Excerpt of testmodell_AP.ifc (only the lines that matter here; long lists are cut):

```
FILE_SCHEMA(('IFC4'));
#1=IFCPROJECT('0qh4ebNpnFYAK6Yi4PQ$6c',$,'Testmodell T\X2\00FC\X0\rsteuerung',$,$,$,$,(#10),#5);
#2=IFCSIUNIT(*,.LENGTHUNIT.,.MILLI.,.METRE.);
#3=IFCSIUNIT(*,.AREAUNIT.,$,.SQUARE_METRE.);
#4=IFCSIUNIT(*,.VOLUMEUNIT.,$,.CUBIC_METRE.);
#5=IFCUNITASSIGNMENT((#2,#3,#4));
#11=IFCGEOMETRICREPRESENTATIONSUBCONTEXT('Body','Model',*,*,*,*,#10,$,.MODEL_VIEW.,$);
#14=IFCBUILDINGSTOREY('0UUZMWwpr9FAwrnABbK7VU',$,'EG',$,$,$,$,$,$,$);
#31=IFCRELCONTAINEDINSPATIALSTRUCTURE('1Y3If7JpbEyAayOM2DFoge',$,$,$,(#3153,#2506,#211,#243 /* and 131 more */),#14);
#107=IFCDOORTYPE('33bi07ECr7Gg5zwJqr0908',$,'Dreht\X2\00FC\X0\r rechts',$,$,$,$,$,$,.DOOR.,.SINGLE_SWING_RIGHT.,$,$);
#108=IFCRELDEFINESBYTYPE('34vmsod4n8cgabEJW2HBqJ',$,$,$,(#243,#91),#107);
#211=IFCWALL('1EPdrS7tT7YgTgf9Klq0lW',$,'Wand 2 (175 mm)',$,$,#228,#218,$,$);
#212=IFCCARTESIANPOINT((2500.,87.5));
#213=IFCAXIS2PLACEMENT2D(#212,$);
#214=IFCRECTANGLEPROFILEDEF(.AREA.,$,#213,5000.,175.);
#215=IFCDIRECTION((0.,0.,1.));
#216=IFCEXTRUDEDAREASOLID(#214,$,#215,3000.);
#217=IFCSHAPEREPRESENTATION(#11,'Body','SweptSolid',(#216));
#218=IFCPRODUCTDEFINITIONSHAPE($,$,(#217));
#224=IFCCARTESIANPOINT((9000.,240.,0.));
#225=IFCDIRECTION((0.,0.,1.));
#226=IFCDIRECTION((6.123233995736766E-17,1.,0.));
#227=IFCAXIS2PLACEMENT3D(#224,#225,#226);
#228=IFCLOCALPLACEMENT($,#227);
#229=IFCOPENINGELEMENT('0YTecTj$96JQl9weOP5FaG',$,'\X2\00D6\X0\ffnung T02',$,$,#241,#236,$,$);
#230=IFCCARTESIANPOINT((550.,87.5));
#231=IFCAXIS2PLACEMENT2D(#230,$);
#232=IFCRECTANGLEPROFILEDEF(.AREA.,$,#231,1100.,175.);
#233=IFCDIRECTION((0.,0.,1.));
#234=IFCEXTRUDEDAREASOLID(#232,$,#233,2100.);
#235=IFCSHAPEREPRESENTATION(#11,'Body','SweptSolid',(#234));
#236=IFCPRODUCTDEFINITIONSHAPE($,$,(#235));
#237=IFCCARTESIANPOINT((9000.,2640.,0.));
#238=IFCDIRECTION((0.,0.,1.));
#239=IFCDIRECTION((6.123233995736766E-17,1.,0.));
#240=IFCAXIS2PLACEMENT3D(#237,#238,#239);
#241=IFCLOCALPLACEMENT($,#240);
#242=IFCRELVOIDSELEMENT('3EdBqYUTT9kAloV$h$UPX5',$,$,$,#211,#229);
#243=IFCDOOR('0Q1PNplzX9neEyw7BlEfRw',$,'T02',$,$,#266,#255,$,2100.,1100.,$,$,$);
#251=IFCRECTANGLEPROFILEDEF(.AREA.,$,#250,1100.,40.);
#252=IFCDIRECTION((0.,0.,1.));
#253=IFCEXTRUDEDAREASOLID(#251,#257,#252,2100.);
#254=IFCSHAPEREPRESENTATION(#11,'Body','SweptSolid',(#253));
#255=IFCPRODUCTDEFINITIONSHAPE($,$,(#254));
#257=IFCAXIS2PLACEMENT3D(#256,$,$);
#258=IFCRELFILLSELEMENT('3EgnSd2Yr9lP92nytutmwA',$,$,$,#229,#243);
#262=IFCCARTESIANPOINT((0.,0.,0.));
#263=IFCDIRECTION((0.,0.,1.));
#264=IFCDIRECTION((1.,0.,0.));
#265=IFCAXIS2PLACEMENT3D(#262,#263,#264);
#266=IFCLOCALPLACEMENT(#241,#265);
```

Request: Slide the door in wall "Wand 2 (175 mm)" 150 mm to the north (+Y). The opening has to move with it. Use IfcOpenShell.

```python
import ifcopenshell
import ifcopenshell.api.geometry
import ifcopenshell.util.placement

model = ifcopenshell.open("testmodell_AP.ifc")

door = model.by_id(243)
opening = door.FillsVoids[0].RelatingOpeningElement
wall = opening.VoidsElements[0].RelatingBuildingElement

wall_matrix = ifcopenshell.util.placement.get_local_placement(wall.ObjectPlacement)
shift = wall_matrix[:3, 0] * 150.0
before = ifcopenshell.util.placement.get_local_placement(door.ObjectPlacement)[:3, 3].copy()

# The door is placed relative to its opening, so it follows when the opening moves.
matrix = ifcopenshell.util.placement.get_local_placement(opening.ObjectPlacement)
matrix[:3, 3] += shift
ifcopenshell.api.geometry.edit_object_placement(
    model, product=opening, matrix=matrix, is_si=False, should_transform_children=True
)

after = ifcopenshell.util.placement.get_local_placement(door.ObjectPlacement)[:3, 3]
print("door moved by", (after - before).round(3) + 0.0)

model.write("testmodell_AP_v2.ifc")
```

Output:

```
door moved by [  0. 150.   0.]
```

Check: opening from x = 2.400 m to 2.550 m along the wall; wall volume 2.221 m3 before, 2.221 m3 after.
